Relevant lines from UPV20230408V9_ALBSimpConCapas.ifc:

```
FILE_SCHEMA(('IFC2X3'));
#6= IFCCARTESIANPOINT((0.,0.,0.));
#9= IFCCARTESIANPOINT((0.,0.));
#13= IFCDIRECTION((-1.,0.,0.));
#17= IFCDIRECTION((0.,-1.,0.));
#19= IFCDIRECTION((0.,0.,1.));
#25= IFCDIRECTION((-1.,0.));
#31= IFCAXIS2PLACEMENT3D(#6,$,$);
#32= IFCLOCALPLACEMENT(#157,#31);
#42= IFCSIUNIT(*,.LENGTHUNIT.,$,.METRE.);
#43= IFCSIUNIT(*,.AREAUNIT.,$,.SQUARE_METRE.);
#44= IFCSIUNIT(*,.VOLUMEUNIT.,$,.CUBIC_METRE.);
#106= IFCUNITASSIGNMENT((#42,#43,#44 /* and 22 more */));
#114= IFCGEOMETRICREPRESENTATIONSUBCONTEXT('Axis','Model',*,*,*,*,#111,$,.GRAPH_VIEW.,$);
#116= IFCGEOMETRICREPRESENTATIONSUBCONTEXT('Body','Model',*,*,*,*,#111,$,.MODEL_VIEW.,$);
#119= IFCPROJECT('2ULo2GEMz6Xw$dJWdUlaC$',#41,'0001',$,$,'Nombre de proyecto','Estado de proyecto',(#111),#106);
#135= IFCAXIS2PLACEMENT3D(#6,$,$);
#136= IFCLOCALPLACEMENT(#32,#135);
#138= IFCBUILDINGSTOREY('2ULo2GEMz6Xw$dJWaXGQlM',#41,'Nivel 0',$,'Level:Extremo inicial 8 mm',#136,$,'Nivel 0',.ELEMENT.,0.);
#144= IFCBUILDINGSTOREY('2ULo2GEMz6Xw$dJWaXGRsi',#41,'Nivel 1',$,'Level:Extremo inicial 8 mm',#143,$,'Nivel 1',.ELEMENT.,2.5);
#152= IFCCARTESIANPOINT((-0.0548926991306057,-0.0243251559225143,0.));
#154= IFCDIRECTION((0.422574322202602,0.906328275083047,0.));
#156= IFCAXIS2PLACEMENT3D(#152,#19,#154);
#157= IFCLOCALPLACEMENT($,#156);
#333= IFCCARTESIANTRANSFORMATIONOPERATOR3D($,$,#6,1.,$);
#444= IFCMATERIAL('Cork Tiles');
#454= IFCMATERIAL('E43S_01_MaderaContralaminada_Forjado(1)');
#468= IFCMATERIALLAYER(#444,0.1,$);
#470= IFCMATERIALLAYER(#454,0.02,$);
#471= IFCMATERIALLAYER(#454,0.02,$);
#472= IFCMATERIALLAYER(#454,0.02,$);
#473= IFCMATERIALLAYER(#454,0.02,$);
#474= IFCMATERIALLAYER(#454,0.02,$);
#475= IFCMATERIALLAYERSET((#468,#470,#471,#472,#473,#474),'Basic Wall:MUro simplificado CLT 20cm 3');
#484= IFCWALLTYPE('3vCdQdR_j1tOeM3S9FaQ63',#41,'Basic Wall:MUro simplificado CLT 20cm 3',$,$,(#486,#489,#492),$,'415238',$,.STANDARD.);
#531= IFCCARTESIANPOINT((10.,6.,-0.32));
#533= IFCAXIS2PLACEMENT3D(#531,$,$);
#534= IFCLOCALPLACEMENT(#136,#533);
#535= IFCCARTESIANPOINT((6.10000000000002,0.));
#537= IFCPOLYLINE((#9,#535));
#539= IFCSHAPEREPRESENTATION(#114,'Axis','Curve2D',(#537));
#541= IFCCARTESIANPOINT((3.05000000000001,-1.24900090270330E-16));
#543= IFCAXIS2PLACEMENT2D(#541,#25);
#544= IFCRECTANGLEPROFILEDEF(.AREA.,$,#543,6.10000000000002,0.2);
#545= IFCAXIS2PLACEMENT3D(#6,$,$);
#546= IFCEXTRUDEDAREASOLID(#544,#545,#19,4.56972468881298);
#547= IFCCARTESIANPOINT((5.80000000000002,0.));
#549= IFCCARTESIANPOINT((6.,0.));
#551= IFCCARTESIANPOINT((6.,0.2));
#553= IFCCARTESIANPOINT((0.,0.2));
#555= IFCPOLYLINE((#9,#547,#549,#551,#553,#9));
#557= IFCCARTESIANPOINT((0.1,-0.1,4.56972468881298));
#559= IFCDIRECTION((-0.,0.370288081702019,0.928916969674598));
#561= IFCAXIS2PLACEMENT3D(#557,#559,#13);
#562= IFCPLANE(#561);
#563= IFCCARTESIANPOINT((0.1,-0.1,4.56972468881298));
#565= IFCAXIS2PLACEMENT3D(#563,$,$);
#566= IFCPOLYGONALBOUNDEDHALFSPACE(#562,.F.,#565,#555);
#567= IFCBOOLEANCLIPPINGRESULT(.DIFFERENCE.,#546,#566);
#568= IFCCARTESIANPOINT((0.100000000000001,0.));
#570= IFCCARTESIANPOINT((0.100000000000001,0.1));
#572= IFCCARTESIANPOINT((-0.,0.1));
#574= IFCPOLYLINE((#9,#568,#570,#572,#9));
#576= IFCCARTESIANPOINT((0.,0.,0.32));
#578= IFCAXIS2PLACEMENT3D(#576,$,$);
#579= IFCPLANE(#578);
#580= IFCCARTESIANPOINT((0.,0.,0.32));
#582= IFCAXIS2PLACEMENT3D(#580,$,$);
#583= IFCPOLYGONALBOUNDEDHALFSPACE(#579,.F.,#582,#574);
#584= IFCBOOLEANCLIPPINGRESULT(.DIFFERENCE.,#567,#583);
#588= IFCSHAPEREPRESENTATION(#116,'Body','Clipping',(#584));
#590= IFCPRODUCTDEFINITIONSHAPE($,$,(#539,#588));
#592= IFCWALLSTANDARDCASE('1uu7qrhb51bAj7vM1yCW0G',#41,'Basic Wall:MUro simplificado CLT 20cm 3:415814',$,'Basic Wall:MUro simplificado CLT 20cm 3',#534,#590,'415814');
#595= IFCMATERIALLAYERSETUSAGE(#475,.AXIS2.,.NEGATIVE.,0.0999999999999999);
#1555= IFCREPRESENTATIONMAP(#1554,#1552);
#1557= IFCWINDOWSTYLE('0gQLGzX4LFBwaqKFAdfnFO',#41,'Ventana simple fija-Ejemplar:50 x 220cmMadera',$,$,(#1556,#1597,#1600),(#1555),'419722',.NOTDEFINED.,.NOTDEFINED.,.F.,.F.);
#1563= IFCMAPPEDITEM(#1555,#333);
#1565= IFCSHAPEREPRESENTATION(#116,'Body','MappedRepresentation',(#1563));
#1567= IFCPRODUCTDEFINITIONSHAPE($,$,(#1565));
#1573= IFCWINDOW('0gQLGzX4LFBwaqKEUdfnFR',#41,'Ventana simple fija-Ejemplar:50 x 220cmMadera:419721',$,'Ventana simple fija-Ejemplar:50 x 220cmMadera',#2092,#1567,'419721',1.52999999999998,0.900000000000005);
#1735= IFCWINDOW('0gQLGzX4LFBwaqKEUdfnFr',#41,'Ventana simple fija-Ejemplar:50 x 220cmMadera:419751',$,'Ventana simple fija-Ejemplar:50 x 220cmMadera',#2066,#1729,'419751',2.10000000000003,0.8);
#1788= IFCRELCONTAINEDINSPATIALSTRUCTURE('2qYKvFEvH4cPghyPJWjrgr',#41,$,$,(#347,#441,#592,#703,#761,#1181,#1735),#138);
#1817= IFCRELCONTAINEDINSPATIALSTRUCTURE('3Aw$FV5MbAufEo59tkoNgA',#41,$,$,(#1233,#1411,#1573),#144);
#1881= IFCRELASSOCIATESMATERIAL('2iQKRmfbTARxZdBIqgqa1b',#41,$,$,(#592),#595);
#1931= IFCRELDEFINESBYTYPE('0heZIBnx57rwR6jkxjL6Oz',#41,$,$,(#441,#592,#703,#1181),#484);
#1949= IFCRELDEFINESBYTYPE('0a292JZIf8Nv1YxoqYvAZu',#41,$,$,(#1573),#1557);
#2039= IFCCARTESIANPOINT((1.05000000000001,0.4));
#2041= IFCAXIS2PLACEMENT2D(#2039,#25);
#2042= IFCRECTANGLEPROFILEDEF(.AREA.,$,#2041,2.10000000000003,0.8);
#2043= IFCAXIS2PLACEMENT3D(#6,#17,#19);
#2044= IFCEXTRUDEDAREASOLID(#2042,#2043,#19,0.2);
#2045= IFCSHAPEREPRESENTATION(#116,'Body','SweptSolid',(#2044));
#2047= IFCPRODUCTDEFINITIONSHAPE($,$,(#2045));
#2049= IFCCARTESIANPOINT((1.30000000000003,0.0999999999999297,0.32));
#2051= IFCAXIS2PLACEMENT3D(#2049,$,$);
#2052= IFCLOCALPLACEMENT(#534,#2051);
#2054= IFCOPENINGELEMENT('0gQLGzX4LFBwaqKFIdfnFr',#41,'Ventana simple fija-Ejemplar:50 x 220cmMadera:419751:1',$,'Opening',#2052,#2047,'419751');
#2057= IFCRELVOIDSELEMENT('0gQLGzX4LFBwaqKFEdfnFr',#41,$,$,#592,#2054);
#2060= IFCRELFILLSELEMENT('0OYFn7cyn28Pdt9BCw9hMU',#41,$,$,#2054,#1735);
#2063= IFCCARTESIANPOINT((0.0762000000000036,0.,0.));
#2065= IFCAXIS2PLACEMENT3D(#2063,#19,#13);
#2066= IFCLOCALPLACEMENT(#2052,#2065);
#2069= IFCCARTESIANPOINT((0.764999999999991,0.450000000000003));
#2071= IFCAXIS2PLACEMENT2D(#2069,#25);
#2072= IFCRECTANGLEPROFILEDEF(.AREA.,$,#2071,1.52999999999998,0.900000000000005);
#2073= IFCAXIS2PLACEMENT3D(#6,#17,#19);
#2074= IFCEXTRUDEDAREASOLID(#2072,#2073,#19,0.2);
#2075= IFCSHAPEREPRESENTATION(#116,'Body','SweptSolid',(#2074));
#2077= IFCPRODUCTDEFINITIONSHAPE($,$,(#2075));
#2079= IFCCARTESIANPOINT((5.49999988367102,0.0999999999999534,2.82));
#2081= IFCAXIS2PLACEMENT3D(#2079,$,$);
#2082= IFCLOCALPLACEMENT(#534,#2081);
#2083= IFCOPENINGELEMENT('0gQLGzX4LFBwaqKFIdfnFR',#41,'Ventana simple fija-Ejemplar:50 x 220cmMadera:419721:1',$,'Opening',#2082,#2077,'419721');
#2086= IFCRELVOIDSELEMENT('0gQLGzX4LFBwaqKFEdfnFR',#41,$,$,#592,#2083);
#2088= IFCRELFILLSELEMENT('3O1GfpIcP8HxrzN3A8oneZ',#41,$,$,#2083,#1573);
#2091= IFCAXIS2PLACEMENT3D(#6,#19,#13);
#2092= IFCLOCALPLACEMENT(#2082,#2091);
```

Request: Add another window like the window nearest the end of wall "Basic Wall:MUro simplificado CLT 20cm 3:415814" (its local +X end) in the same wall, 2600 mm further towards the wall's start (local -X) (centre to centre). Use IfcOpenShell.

```python
import ifcopenshell
import ifcopenshell.api.feature
import ifcopenshell.api.geometry
import ifcopenshell.api.root
import ifcopenshell.geom
import ifcopenshell.util.element
import ifcopenshell.util.placement
import ifcopenshell.util.shape
import ifcopenshell.util.unit

model = ifcopenshell.open("UPV20230408V9_ALBSimpConCapas.ifc")
unit_scale = ifcopenshell.util.unit.calculate_unit_scale(model)
settings = ifcopenshell.geom.settings()


def volume(element):
    """Net volume in cubic metres, openings subtracted."""
    shape = ifcopenshell.geom.create_shape(settings, element)
    return ifcopenshell.util.shape.get_volume(shape.geometry)


def reuse_history(source, copy):
    """copy_class also copies each property set's owner history, people and application; keep the originals."""
    for rel in copy.IsDefinedBy:
        if rel.is_a("IfcRelDefinesByProperties") and (history := rel.RelatingPropertyDefinition.OwnerHistory):
            rel.RelatingPropertyDefinition.OwnerHistory = source.OwnerHistory
            ifcopenshell.util.element.remove_deep2(model, history)


window = model.by_guid("0gQLGzX4LFBwaqKEUdfnFR")
opening = window.FillsVoids[0].RelatingOpeningElement
wall = opening.VoidsElements[0].RelatingBuildingElement
before = volume(wall)
shift = ifcopenshell.util.placement.get_local_placement(wall.ObjectPlacement)[:3, 0] * -2.6 / unit_scale

# copy_class copies the void relationship, type, container and properties, but no geometry.
new_opening = ifcopenshell.api.root.copy_class(model, product=opening)
new_opening.Representation = ifcopenshell.util.element.copy_deep(
    model, opening.Representation, exclude=["IfcGeometricRepresentationContext", "IfcRepresentationMap"]
)
new_opening.Name = "Ventana simple fija-Ejemplar:50 x 220cmMadera"
new_opening.Tag = None
new_window = ifcopenshell.api.root.copy_class(model, product=window)
new_window.Representation = ifcopenshell.util.element.copy_deep(
    model, window.Representation, exclude=["IfcGeometricRepresentationContext", "IfcRepresentationMap"]
)
new_window.Name = "Ventana simple fija-Ejemplar:50 x 220cmMadera"
new_window.Tag = None
reuse_history(window, new_window)
fills = ifcopenshell.api.feature.add_filling(model, opening=new_opening, element=new_window)
fills.OwnerHistory = new_window.OwnerHistory  # required in IFC2X3

for old, new in ((opening, new_opening), (window, new_window)):
    matrix = ifcopenshell.util.placement.get_local_placement(old.ObjectPlacement)
    matrix[:3, 3] += shift
    ifcopenshell.api.geometry.edit_object_placement(model, product=new, matrix=matrix, is_si=False)

after = volume(wall)

print(f"wall volume {before:.3f} -> {after:.3f} m3")

model.write("UPV20230408V9_ALBSimpConCapas_updated.ifc")
```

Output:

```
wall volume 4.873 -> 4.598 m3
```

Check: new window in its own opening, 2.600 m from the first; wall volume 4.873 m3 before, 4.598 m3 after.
